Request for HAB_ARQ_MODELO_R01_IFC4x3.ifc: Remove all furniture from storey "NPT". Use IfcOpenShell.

First a look at what the model holds.

```python
import ifcopenshell
import ifcopenshell.util.element

model = ifcopenshell.open("HAB_ARQ_MODELO_R01_IFC4x3.ifc")
print(model.schema)
storey = next(s for s in model.by_type("IfcBuildingStorey") if s.Name == "NPT")
furniture = [e for e in ifcopenshell.util.element.get_decomposition(storey) if e.is_a("IfcFurnishingElement")]
seen = {}
for e in furniture:
    element_type = ifcopenshell.util.element.get_type(e)
    name = element_type.Name if element_type not in (None, e) else None
    seen[name] = seen.get(name, 0) + 1
for name, count in sorted(seen.items(), key=str):
    print(count, "x", name)
```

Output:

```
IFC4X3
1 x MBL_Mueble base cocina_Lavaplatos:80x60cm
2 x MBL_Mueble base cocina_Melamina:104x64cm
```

```python
import ifcopenshell
import ifcopenshell.api.root
import ifcopenshell.util.element

model = ifcopenshell.open("HAB_ARQ_MODELO_R01_IFC4x3.ifc")

storey = next(s for s in model.by_type("IfcBuildingStorey") if s.Name == "NPT")
furniture = [e for e in ifcopenshell.util.element.get_decomposition(storey) if e.is_a("IfcFurnishingElement")]

for e in furniture:
    ifcopenshell.api.root.remove_product(model, product=e)
print(len(furniture), "removed")

model.write("HAB_ARQ_MODELO_R01_IFC4x3_v2.ifc")
```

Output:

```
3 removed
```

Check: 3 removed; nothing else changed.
